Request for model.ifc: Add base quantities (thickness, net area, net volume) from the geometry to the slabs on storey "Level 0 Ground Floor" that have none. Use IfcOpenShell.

First a look at what the model holds.

```python
import ifcopenshell
import ifcopenshell.util.element
import ifcopenshell.util.unit

model = ifcopenshell.open("model.ifc")
print(model.schema)
for unit_type in ("LENGTHUNIT", "AREAUNIT", "VOLUMEUNIT"):
    print(unit_type, ifcopenshell.util.unit.calculate_unit_scale(model, unit_type))
storey = next(s for s in model.by_type("IfcBuildingStorey") if s.Name == "Level 0 Ground Floor")
slabs = [e for e in ifcopenshell.util.element.get_decomposition(storey) if e.is_a("IfcSlab")]
for e in sorted(slabs, key=lambda e: e.id()):
    print(e.id(), e.is_a(), e.Name, list(ifcopenshell.util.element.get_psets(e, qtos_only=True)), sep=" | ")
```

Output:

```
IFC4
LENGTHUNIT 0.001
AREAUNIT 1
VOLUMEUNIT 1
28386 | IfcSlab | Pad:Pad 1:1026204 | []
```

```python
import ifcopenshell
import ifcopenshell.api.pset
import ifcopenshell.geom
import ifcopenshell.util.element
import ifcopenshell.util.shape
import ifcopenshell.util.unit

model = ifcopenshell.open("model.ifc")
unit_scale = ifcopenshell.util.unit.calculate_unit_scale(model)
area_scale = ifcopenshell.util.unit.calculate_unit_scale(model, "AREAUNIT")
volume_scale = ifcopenshell.util.unit.calculate_unit_scale(model, "VOLUMEUNIT")
settings = ifcopenshell.geom.settings()

storey = next(s for s in model.by_type("IfcBuildingStorey") if s.Name == "Level 0 Ground Floor")
slabs = [e for e in ifcopenshell.util.element.get_decomposition(storey) if e.is_a("IfcSlab")]

for e in sorted(slabs, key=lambda e: e.id()):
    if ifcopenshell.util.element.get_psets(e, qtos_only=True, should_inherit=False):
        continue
    # Geometry comes back in metres, in the element's own axes.
    shape = ifcopenshell.geom.create_shape(settings, e)
    values = {
        "Width": ifcopenshell.util.shape.get_z(shape.geometry) / unit_scale,
        "NetArea": ifcopenshell.util.shape.get_footprint_area(shape.geometry) / area_scale,
        "NetVolume": ifcopenshell.util.shape.get_volume(shape.geometry) / volume_scale,
    }
    qto = ifcopenshell.api.pset.add_qto(model, product=e, name="Qto_SlabBaseQuantities")
    ifcopenshell.api.pset.edit_qto(model, qto=qto, properties=values)
    print(e.id(), {k: round(v, 3) for k, v in values.items()})

model.write("model-out.ifc")
```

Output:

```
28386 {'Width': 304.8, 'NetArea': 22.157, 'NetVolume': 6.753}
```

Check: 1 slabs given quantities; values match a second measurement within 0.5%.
